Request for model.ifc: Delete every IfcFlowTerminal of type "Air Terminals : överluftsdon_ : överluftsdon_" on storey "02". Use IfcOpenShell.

First a look at what the model holds.

```python
import ifcopenshell
import ifcopenshell.util.element

model = ifcopenshell.open("model.ifc")
print(model.schema)
storey = next(s for s in model.by_type("IfcBuildingStorey") if s.Name == "02")
terminals = [e for e in ifcopenshell.util.element.get_decomposition(storey) if e.is_a("IfcFlowTerminal")]
seen = {}
for e in terminals:
    element_type = ifcopenshell.util.element.get_type(e)
    name = element_type.Name if element_type not in (None, e) else None
    seen[name] = seen.get(name, 0) + 1
for name, count in sorted(seen.items(), key=str):
    print(count, "x", name)
```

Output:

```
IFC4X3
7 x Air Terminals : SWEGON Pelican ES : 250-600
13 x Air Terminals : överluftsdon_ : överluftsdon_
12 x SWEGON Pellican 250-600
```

```python
import ifcopenshell
import ifcopenshell.api.root
import ifcopenshell.util.element

model = ifcopenshell.open("model.ifc")

storey = next(s for s in model.by_type("IfcBuildingStorey") if s.Name == "02")
terminals = [e for e in ifcopenshell.util.element.get_decomposition(storey) if e.is_a("IfcFlowTerminal")]
targets = [e for e in terminals if (t := ifcopenshell.util.element.get_type(e)) not in (None, e) and t.Name == "Air Terminals : överluftsdon_ : överluftsdon_"]

for e in targets:
    ifcopenshell.api.root.remove_product(model, product=e)
print(len(targets), "removed")

model.write("model_updated.ifc")
```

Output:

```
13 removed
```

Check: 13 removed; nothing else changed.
